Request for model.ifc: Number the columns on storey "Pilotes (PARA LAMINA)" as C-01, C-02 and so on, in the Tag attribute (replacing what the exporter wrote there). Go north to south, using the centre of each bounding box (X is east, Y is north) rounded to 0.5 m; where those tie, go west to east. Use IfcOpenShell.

First a look at what the model holds.

```python
import ifcopenshell
import ifcopenshell.util.element
import ifcopenshell.util.placement

model = ifcopenshell.open("model.ifc")
print(model.schema)
storey = next(s for s in model.by_type("IfcBuildingStorey") if s.Name == "Pilotes (PARA LAMINA)")
columns = [e for e in ifcopenshell.util.element.get_decomposition(storey) if e.is_a("IfcColumn")]
for e in sorted(columns, key=lambda e: e.id()):
    origin = ifcopenshell.util.placement.get_local_placement(e.ObjectPlacement)[:3, 3]
    print(e.id(), e.Tag, e.Name, origin.round(2) + 0.0, sep=" | ")
```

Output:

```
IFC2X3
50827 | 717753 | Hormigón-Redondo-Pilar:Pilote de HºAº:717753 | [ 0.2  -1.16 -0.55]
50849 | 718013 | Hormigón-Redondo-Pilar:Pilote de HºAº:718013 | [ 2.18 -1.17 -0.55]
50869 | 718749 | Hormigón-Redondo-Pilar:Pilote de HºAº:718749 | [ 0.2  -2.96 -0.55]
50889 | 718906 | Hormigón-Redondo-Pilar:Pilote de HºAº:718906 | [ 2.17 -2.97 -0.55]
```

```python
import ifcopenshell
import ifcopenshell.geom
import ifcopenshell.util.element
import ifcopenshell.util.shape

model = ifcopenshell.open("model.ifc")
settings = ifcopenshell.geom.settings()
settings.set("use-world-coords", True)


def centre(element):
    shape = ifcopenshell.geom.create_shape(settings, element)
    return ifcopenshell.util.shape.get_bbox_centroid(shape.geometry)


storey = next(s for s in model.by_type("IfcBuildingStorey") if s.Name == "Pilotes (PARA LAMINA)")
columns = [e for e in ifcopenshell.util.element.get_decomposition(storey) if e.is_a("IfcColumn")]

# Insertion points can sit at a corner or the storey origin, so sort by the geometry (in metres).
centres = {e: centre(e) for e in columns}
columns.sort(key=lambda e: (-round(centres[e][1] / 0.5), centres[e][0]))

for i, e in enumerate(columns, start=1):
    number = f"C-{i:02d}"
    e.Tag = number
    print(e.id(), number)

model.write("model-out.ifc")
```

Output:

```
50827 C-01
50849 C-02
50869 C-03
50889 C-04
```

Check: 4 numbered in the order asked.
